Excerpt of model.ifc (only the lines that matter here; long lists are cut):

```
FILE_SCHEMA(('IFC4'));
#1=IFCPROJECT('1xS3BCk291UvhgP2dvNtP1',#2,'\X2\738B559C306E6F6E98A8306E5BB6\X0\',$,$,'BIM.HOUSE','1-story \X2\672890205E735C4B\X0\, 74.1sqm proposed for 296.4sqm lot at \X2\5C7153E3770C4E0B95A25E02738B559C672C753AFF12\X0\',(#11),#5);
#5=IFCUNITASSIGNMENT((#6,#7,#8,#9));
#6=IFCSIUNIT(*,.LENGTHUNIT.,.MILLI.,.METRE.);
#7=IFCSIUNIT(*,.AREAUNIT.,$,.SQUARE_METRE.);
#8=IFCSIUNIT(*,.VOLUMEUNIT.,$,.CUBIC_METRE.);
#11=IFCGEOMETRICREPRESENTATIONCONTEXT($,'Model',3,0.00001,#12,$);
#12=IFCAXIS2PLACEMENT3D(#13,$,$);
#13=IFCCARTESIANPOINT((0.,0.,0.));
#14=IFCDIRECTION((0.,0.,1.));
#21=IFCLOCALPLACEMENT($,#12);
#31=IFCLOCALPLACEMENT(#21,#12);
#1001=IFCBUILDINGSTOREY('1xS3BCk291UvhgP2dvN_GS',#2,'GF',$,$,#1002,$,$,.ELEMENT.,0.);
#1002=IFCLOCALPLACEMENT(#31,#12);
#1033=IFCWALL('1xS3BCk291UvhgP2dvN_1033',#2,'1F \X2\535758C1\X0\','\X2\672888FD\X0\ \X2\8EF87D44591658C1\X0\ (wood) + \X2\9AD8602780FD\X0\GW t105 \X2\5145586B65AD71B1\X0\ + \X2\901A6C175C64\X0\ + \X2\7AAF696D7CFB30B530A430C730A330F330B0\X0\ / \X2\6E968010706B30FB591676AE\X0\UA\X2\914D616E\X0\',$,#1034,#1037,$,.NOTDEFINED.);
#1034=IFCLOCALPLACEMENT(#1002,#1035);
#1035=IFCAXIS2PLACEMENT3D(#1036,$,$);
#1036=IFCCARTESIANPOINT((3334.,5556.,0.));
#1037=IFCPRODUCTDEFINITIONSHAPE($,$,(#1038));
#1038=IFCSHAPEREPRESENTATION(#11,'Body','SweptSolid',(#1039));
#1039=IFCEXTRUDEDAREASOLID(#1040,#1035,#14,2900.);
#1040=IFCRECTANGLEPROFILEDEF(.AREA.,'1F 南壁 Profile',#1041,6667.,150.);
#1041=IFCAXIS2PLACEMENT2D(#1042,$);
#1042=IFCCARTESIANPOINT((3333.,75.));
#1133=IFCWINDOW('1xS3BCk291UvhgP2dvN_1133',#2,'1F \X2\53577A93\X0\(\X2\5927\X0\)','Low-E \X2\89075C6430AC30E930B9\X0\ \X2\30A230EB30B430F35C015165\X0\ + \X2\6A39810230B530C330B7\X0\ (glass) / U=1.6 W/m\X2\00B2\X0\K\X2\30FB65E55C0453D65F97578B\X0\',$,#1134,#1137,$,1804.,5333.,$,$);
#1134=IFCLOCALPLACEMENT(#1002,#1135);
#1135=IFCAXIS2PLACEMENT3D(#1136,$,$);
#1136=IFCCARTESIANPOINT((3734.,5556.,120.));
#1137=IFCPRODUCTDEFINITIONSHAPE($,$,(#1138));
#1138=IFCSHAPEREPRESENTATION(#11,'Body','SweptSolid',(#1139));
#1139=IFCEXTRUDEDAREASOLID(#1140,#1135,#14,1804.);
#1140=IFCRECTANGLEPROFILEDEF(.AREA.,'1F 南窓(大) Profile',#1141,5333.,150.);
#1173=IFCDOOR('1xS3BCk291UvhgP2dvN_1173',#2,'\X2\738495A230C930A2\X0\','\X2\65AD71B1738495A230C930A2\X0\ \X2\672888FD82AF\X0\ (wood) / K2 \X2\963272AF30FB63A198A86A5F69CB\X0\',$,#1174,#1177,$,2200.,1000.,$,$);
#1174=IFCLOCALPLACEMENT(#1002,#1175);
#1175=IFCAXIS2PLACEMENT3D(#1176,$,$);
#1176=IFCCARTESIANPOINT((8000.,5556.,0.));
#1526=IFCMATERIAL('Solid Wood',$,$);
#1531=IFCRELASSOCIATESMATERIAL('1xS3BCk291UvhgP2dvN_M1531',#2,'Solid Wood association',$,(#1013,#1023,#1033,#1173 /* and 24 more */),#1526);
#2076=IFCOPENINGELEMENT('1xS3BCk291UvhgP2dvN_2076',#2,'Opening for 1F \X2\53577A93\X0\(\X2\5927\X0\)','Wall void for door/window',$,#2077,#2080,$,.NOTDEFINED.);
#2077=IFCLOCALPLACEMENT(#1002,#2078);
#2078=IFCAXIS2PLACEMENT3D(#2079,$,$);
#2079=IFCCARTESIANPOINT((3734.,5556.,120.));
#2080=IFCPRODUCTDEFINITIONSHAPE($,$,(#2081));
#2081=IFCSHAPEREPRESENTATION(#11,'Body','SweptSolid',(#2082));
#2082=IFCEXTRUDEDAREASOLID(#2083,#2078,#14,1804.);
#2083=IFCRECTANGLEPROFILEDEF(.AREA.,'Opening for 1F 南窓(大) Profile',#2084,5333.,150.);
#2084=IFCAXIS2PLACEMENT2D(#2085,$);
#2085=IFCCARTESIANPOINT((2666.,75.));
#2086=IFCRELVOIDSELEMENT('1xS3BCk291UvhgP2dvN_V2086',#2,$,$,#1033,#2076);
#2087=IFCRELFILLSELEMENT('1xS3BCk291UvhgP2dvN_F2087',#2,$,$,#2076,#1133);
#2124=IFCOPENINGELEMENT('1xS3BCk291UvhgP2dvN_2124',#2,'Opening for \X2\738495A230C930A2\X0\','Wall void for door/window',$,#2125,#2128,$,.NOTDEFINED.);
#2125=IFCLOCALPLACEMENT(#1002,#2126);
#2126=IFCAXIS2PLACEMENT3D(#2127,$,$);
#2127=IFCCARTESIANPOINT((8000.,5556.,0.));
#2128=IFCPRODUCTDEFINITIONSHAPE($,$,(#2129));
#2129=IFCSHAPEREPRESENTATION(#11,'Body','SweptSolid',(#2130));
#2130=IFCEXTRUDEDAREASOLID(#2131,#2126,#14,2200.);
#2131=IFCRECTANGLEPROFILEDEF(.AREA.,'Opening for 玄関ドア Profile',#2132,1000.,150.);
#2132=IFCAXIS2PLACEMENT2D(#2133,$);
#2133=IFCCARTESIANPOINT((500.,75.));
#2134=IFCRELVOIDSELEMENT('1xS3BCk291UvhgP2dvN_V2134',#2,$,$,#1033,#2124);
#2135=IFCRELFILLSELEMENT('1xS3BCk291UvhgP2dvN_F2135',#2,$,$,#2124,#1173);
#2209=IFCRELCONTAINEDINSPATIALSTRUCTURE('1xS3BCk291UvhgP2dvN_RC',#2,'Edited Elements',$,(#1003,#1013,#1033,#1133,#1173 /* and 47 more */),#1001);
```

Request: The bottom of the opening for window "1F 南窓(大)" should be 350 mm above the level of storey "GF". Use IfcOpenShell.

```python
import numpy as np
import ifcopenshell
import ifcopenshell.api.geometry
import ifcopenshell.geom
import ifcopenshell.util.element
import ifcopenshell.util.placement
import ifcopenshell.util.shape
import ifcopenshell.util.unit

model = ifcopenshell.open("model.ifc")
unit_scale = ifcopenshell.util.unit.calculate_unit_scale(model)

window = model.by_id(1133)
opening = window.FillsVoids[0].RelatingOpeningElement
storey = ifcopenshell.util.element.get_container(window, ifc_class="IfcBuildingStorey")
level = ifcopenshell.util.placement.get_local_placement(storey.ObjectPlacement)[2, 3]

# The opening's origin need not be at the sill, so measure its lowest point.
shape = ifcopenshell.geom.create_shape(ifcopenshell.geom.settings(), opening)
bottom = ifcopenshell.util.shape.get_shape_bottom_elevation(shape, shape.geometry) / unit_scale
dz = level + 350.0 - bottom

shift = np.array([0.0, 0.0, dz])
# The window is not placed relative to its opening, so move both.
for product in (opening, window):
    matrix = ifcopenshell.util.placement.get_local_placement(product.ObjectPlacement)
    matrix[:3, 3] += shift
    ifcopenshell.api.geometry.edit_object_placement(model, product=product, matrix=matrix, is_si=False)

print(f"moved by {dz * unit_scale:+.3f} m")

model.write("model_v2.ifc")
```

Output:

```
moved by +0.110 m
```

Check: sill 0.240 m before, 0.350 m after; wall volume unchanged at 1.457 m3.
